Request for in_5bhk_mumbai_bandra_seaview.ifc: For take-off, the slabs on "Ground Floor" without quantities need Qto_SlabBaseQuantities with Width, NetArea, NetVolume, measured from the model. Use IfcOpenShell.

First a look at what the model holds.

```python
import ifcopenshell
import ifcopenshell.util.element
import ifcopenshell.util.unit

model = ifcopenshell.open("in_5bhk_mumbai_bandra_seaview.ifc")
print(model.schema)
for unit_type in ("LENGTHUNIT", "AREAUNIT", "VOLUMEUNIT"):
    print(unit_type, ifcopenshell.util.unit.calculate_unit_scale(model, unit_type))
storey = next(s for s in model.by_type("IfcBuildingStorey") if s.Name == "Ground Floor")
slabs = [e for e in ifcopenshell.util.element.get_decomposition(storey) if e.is_a("IfcSlab")]
for e in sorted(slabs, key=lambda e: e.id()):
    print(e.id(), e.is_a(), e.Name, list(ifcopenshell.util.element.get_psets(e, qtos_only=True)), sep=" | ")
```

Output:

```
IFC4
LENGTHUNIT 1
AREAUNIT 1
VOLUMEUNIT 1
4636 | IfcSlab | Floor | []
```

```python
import ifcopenshell
import ifcopenshell.api.pset
import ifcopenshell.geom
import ifcopenshell.util.element
import ifcopenshell.util.shape
import ifcopenshell.util.unit

model = ifcopenshell.open("in_5bhk_mumbai_bandra_seaview.ifc")
unit_scale = ifcopenshell.util.unit.calculate_unit_scale(model)
area_scale = ifcopenshell.util.unit.calculate_unit_scale(model, "AREAUNIT")
volume_scale = ifcopenshell.util.unit.calculate_unit_scale(model, "VOLUMEUNIT")
settings = ifcopenshell.geom.settings()

storey = next(s for s in model.by_type("IfcBuildingStorey") if s.Name == "Ground Floor")
slabs = [e for e in ifcopenshell.util.element.get_decomposition(storey) if e.is_a("IfcSlab")]

for e in sorted(slabs, key=lambda e: e.id()):
    if ifcopenshell.util.element.get_psets(e, qtos_only=True, should_inherit=False):
        continue
    # Geometry comes back in metres, in the element's own axes.
    shape = ifcopenshell.geom.create_shape(settings, e)
    values = {
        "Width": ifcopenshell.util.shape.get_z(shape.geometry) / unit_scale,
        "NetArea": ifcopenshell.util.shape.get_footprint_area(shape.geometry) / area_scale,
        "NetVolume": ifcopenshell.util.shape.get_volume(shape.geometry) / volume_scale,
    }
    qto = ifcopenshell.api.pset.add_qto(model, product=e, name="Qto_SlabBaseQuantities")
    ifcopenshell.api.pset.edit_qto(model, qto=qto, properties=values)
    print(e.id(), {k: round(v, 3) for k, v in values.items()})

model.write("in_5bhk_mumbai_bandra_seaview-out.ifc")
```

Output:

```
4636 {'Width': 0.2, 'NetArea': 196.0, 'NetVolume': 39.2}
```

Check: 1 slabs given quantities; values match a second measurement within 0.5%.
